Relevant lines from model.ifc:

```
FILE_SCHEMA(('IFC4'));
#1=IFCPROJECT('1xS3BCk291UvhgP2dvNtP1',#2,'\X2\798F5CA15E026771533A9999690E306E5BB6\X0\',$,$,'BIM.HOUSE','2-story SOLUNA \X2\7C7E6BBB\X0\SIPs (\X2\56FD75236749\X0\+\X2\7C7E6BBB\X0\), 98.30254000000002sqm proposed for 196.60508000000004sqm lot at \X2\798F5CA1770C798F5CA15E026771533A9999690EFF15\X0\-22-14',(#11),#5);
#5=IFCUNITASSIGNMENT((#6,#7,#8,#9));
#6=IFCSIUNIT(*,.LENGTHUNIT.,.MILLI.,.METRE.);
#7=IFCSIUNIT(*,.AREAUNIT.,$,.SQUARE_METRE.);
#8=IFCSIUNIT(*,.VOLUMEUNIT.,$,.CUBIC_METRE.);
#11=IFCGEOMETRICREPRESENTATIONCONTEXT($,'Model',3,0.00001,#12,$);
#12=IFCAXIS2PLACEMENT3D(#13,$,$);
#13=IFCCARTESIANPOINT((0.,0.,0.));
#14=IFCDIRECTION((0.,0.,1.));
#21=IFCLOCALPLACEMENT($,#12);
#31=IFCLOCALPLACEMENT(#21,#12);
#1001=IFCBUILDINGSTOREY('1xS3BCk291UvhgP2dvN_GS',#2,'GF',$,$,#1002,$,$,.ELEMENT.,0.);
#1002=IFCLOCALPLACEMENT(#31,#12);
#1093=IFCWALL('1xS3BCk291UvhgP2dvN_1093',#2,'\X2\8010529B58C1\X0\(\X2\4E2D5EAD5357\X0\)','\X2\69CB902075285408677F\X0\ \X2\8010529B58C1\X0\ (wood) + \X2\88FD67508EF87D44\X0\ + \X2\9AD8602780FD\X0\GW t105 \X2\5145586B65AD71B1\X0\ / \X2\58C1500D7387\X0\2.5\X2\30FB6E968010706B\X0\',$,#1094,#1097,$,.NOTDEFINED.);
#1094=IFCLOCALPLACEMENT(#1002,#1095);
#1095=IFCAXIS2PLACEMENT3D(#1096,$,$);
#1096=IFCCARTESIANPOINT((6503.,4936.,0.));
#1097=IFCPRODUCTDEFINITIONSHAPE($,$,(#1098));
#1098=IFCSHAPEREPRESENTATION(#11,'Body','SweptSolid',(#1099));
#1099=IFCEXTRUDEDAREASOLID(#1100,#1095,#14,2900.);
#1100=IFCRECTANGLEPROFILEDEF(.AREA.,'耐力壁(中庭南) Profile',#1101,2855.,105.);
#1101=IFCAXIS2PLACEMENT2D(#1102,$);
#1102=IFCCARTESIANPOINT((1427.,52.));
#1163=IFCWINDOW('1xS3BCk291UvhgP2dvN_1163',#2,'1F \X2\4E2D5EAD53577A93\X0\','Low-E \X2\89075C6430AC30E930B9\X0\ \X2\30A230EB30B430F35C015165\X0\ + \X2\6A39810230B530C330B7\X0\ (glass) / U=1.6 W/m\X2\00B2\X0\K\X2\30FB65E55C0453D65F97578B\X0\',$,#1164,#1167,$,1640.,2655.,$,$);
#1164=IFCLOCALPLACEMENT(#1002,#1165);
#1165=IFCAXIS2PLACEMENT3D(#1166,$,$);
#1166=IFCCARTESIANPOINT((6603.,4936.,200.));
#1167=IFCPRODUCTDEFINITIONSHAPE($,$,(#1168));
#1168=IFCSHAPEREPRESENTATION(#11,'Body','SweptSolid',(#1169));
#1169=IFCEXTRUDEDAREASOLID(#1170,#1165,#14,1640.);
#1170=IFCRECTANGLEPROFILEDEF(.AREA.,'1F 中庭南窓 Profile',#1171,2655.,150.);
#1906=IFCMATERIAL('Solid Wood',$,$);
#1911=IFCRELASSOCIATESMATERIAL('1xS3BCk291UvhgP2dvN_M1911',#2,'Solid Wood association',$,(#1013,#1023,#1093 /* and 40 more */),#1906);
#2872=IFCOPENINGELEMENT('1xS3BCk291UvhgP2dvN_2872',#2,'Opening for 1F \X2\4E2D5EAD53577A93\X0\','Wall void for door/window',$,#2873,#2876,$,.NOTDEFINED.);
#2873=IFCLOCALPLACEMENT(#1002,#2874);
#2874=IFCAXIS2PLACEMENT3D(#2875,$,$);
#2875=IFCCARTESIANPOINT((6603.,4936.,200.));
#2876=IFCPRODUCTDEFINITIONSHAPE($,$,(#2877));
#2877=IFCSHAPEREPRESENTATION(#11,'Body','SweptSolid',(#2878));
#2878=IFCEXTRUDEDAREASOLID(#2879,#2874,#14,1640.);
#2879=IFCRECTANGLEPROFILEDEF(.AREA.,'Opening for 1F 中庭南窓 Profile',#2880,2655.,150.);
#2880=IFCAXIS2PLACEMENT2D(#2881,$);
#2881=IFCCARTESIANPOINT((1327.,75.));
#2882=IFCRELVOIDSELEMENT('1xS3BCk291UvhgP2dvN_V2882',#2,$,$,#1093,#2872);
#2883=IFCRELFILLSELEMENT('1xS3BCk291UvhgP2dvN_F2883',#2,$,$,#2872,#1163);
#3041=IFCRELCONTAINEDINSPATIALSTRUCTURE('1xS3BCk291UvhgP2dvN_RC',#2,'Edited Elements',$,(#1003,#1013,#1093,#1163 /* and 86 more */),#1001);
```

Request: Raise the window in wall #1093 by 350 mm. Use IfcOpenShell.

```python
import numpy as np
import ifcopenshell
import ifcopenshell.api.geometry
import ifcopenshell.util.placement
import ifcopenshell.util.unit

model = ifcopenshell.open("model.ifc")
unit_scale = ifcopenshell.util.unit.calculate_unit_scale(model)

window = model.by_guid("1xS3BCk291UvhgP2dvN_1163")
opening = window.FillsVoids[0].RelatingOpeningElement
dz = 0.35 / unit_scale

shift = np.array([0.0, 0.0, dz])
# The window is not placed relative to its opening, so move both.
for product in (opening, window):
    matrix = ifcopenshell.util.placement.get_local_placement(product.ObjectPlacement)
    matrix[:3, 3] += shift
    ifcopenshell.api.geometry.edit_object_placement(model, product=product, matrix=matrix, is_si=False)

print(f"moved by {dz * unit_scale:+.3f} m")

model.write("model_v2.ifc")
```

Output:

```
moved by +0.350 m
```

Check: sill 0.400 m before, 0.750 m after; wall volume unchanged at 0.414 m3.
